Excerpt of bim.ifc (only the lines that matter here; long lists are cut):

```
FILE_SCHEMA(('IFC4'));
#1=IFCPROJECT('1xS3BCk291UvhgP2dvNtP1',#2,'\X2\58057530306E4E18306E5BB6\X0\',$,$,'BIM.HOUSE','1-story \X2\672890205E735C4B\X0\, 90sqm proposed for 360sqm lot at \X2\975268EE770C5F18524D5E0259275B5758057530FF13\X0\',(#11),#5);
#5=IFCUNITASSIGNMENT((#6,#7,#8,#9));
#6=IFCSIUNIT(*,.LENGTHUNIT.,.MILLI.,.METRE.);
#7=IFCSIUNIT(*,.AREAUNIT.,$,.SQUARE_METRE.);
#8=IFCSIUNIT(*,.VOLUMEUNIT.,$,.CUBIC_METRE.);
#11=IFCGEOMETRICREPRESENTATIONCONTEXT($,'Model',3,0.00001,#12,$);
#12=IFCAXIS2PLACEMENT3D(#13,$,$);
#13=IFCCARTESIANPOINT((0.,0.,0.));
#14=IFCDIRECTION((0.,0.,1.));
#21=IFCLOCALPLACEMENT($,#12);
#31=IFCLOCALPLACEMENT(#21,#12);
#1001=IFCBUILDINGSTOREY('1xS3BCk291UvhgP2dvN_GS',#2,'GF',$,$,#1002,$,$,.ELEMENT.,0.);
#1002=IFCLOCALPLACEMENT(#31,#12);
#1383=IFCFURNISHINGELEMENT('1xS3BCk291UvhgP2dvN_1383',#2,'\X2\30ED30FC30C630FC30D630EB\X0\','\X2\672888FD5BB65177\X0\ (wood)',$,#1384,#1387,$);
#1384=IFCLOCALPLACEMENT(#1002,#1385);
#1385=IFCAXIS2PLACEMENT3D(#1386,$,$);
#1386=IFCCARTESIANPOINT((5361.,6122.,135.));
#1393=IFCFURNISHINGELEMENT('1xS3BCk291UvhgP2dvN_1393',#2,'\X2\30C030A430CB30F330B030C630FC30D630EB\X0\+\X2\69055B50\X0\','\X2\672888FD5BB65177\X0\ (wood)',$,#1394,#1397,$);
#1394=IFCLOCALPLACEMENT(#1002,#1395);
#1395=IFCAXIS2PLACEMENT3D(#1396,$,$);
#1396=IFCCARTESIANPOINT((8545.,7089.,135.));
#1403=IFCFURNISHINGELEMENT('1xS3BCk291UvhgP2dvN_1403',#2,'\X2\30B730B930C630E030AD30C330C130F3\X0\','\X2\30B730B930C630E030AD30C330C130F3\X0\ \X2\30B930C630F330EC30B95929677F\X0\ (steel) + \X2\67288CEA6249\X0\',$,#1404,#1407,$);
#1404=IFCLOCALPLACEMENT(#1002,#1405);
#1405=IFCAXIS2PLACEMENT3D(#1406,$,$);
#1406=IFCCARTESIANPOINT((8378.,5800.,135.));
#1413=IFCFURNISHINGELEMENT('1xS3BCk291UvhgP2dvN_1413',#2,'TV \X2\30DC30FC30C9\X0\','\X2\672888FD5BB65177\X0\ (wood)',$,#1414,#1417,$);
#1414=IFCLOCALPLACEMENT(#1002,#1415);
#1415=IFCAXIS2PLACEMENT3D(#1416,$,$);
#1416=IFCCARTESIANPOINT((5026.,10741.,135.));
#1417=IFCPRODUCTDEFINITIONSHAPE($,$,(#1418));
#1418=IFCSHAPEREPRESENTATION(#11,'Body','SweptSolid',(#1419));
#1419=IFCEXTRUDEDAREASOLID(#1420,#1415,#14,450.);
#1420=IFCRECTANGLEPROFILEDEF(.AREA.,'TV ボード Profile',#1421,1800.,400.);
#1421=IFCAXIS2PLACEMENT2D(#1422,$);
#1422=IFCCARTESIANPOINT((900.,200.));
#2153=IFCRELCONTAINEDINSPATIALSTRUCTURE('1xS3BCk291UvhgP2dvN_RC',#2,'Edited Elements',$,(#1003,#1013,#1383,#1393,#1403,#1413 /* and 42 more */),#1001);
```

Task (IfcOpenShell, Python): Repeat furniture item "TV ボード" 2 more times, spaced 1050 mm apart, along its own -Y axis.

```python
import ifcopenshell
import ifcopenshell.api.geometry
import ifcopenshell.api.root
import ifcopenshell.util.element
import ifcopenshell.util.placement

model = ifcopenshell.open("bim.ifc")


def reuse_history(source, copy):
    """copy_class also copies each property set's owner history, people and application; keep the originals."""
    for rel in copy.IsDefinedBy:
        if rel.is_a("IfcRelDefinesByProperties") and (history := rel.RelatingPropertyDefinition.OwnerHistory):
            rel.RelatingPropertyDefinition.OwnerHistory = source.OwnerHistory
            ifcopenshell.util.element.remove_deep2(model, history)


source = model.by_guid("1xS3BCk291UvhgP2dvN_1413")
base = ifcopenshell.util.placement.get_local_placement(source.ObjectPlacement)
step = -base[:3, 1] * 1050.0

for i in range(1, 3):
    copy = ifcopenshell.api.root.copy_class(model, product=source)
    copy.Representation = ifcopenshell.util.element.copy_deep(
        model, source.Representation, exclude=["IfcGeometricRepresentationContext", "IfcRepresentationMap"]
    )
    reuse_history(source, copy)
    matrix = base.copy()
    matrix[:3, 3] += i * step
    print("added at", matrix[:3, 3].round(3) + 0.0)
    ifcopenshell.api.geometry.edit_object_placement(model, product=copy, matrix=matrix, is_si=False)

model.write("bim_v2.ifc")
```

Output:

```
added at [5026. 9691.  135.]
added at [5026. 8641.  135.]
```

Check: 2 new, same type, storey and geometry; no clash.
